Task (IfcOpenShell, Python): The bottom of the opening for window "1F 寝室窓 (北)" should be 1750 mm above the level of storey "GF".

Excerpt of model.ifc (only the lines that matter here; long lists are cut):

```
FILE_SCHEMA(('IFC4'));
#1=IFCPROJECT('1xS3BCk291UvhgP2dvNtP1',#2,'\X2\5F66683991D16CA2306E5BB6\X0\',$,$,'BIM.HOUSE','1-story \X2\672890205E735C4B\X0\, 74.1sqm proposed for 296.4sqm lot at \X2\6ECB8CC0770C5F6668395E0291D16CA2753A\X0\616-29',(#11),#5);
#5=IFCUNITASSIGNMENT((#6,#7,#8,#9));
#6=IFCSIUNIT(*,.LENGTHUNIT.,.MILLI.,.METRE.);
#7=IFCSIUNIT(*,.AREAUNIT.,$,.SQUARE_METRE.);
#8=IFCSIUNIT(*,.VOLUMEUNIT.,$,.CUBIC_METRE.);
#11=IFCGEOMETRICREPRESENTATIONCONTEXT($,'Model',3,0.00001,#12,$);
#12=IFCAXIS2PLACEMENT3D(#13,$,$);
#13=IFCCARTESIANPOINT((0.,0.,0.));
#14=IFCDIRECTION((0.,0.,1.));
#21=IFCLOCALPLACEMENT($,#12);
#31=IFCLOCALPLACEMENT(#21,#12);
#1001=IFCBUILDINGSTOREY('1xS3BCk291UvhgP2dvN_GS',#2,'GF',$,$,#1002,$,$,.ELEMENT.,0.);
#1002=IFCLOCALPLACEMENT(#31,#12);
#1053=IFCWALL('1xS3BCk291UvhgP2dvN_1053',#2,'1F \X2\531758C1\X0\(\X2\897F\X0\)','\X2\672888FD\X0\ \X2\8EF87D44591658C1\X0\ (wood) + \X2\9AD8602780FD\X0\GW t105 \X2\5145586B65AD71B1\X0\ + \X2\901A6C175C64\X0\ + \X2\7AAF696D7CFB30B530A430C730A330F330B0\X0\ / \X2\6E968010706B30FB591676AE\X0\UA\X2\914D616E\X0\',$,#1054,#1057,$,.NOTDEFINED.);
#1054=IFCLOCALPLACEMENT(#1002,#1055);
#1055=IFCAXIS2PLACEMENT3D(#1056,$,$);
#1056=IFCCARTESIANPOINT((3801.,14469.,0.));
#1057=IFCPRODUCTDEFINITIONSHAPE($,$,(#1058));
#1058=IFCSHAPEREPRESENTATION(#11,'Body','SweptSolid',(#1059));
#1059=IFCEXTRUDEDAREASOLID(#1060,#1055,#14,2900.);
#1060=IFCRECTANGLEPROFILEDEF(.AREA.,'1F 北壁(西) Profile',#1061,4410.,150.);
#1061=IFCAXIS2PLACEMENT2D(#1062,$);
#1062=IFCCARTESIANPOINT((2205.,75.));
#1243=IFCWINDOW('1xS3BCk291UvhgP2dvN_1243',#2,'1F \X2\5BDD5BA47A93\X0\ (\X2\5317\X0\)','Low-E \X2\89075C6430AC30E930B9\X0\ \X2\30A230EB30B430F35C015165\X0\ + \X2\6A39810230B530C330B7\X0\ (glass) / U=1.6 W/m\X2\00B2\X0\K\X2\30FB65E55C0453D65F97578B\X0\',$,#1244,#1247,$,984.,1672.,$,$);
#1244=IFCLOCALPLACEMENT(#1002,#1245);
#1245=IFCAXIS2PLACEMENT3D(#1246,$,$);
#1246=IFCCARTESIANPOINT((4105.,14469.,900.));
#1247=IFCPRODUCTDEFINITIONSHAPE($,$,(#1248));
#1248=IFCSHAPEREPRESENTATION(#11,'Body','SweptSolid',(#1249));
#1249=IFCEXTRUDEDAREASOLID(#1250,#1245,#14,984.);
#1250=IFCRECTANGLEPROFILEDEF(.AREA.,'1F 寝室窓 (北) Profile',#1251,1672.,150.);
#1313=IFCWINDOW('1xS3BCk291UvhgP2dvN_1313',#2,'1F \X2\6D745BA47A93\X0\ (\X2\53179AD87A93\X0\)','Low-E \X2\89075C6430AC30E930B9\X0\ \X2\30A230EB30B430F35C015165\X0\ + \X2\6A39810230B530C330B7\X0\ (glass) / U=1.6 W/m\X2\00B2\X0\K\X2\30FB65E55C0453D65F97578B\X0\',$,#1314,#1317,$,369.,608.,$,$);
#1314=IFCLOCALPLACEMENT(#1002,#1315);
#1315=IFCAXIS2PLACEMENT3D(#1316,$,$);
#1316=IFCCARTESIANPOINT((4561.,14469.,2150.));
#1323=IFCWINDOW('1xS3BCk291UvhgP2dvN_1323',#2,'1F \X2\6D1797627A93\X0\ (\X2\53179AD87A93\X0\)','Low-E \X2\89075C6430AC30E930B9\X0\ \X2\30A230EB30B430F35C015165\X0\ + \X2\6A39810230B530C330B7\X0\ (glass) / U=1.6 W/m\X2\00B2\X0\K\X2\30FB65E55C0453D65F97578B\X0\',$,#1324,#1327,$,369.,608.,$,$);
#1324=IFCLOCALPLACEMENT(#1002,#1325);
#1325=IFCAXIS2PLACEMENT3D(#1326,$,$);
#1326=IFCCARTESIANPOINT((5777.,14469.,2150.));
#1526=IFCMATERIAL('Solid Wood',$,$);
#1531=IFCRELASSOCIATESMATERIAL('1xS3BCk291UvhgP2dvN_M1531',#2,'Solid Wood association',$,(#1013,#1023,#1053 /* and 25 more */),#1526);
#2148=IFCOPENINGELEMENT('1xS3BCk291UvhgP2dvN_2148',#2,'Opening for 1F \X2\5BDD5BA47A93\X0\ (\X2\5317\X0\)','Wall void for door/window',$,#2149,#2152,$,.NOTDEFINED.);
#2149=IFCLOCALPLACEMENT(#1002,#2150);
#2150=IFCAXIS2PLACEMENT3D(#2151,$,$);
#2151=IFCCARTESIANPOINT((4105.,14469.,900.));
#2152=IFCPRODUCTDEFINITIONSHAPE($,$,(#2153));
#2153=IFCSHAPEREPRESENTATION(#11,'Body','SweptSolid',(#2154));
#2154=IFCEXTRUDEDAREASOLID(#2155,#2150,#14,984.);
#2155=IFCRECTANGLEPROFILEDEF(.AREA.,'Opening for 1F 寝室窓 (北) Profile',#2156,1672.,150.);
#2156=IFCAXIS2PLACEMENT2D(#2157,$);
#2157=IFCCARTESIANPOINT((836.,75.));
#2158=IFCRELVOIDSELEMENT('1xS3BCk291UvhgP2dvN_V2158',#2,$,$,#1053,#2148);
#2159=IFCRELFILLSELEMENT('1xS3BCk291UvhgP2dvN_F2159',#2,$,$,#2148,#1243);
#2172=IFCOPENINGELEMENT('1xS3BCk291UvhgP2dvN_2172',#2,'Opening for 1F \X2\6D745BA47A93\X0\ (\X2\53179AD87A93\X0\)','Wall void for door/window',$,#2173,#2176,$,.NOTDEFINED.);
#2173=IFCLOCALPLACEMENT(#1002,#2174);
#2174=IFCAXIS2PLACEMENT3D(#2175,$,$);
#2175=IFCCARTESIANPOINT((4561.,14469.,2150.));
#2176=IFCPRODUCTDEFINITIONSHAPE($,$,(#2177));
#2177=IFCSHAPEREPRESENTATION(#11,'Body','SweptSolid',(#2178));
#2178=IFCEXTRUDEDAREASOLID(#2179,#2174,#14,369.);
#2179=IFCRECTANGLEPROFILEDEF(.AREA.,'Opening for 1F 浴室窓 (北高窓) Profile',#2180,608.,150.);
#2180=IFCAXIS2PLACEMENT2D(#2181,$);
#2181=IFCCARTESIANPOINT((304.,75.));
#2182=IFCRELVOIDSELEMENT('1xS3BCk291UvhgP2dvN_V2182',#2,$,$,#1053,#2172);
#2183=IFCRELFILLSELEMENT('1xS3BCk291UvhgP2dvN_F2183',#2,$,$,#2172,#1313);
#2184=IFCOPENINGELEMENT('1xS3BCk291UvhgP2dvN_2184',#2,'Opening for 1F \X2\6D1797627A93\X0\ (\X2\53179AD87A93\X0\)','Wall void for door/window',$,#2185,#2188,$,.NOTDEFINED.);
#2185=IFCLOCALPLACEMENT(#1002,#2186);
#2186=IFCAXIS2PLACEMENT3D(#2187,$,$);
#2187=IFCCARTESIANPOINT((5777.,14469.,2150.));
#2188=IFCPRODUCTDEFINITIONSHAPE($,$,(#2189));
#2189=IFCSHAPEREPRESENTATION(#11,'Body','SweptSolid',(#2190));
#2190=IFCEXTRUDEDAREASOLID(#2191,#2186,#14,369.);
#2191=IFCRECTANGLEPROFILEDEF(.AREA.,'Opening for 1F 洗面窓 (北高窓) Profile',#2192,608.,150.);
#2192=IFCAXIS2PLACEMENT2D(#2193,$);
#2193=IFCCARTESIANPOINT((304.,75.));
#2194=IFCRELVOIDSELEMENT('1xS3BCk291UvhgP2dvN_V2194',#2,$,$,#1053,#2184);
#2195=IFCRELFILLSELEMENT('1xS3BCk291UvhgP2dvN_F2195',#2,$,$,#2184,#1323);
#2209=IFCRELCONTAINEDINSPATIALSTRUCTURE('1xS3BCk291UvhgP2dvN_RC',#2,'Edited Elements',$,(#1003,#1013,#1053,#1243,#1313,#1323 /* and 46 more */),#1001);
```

```python
import numpy as np
import ifcopenshell
import ifcopenshell.api.geometry
import ifcopenshell.geom
import ifcopenshell.util.element
import ifcopenshell.util.placement
import ifcopenshell.util.shape
import ifcopenshell.util.unit

model = ifcopenshell.open("model.ifc")
unit_scale = ifcopenshell.util.unit.calculate_unit_scale(model)

window = model.by_guid("1xS3BCk291UvhgP2dvN_1243")
opening = window.FillsVoids[0].RelatingOpeningElement
storey = ifcopenshell.util.element.get_container(window, ifc_class="IfcBuildingStorey")
level = ifcopenshell.util.placement.get_local_placement(storey.ObjectPlacement)[2, 3]

# The opening's origin need not be at the sill, so measure its lowest point.
shape = ifcopenshell.geom.create_shape(ifcopenshell.geom.settings(), opening)
bottom = ifcopenshell.util.shape.get_shape_bottom_elevation(shape, shape.geometry) / unit_scale
dz = level + 1750.0 - bottom

shift = np.array([0.0, 0.0, dz])
# The window is not placed relative to its opening, so move both.
for product in (opening, window):
    matrix = ifcopenshell.util.placement.get_local_placement(product.ObjectPlacement)
    matrix[:3, 3] += shift
    ifcopenshell.api.geometry.edit_object_placement(model, product=product, matrix=matrix, is_si=False)

print(f"moved by {dz * unit_scale:+.3f} m")

model.write("model-out.ifc")
```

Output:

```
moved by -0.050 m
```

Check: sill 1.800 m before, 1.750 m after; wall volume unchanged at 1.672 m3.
